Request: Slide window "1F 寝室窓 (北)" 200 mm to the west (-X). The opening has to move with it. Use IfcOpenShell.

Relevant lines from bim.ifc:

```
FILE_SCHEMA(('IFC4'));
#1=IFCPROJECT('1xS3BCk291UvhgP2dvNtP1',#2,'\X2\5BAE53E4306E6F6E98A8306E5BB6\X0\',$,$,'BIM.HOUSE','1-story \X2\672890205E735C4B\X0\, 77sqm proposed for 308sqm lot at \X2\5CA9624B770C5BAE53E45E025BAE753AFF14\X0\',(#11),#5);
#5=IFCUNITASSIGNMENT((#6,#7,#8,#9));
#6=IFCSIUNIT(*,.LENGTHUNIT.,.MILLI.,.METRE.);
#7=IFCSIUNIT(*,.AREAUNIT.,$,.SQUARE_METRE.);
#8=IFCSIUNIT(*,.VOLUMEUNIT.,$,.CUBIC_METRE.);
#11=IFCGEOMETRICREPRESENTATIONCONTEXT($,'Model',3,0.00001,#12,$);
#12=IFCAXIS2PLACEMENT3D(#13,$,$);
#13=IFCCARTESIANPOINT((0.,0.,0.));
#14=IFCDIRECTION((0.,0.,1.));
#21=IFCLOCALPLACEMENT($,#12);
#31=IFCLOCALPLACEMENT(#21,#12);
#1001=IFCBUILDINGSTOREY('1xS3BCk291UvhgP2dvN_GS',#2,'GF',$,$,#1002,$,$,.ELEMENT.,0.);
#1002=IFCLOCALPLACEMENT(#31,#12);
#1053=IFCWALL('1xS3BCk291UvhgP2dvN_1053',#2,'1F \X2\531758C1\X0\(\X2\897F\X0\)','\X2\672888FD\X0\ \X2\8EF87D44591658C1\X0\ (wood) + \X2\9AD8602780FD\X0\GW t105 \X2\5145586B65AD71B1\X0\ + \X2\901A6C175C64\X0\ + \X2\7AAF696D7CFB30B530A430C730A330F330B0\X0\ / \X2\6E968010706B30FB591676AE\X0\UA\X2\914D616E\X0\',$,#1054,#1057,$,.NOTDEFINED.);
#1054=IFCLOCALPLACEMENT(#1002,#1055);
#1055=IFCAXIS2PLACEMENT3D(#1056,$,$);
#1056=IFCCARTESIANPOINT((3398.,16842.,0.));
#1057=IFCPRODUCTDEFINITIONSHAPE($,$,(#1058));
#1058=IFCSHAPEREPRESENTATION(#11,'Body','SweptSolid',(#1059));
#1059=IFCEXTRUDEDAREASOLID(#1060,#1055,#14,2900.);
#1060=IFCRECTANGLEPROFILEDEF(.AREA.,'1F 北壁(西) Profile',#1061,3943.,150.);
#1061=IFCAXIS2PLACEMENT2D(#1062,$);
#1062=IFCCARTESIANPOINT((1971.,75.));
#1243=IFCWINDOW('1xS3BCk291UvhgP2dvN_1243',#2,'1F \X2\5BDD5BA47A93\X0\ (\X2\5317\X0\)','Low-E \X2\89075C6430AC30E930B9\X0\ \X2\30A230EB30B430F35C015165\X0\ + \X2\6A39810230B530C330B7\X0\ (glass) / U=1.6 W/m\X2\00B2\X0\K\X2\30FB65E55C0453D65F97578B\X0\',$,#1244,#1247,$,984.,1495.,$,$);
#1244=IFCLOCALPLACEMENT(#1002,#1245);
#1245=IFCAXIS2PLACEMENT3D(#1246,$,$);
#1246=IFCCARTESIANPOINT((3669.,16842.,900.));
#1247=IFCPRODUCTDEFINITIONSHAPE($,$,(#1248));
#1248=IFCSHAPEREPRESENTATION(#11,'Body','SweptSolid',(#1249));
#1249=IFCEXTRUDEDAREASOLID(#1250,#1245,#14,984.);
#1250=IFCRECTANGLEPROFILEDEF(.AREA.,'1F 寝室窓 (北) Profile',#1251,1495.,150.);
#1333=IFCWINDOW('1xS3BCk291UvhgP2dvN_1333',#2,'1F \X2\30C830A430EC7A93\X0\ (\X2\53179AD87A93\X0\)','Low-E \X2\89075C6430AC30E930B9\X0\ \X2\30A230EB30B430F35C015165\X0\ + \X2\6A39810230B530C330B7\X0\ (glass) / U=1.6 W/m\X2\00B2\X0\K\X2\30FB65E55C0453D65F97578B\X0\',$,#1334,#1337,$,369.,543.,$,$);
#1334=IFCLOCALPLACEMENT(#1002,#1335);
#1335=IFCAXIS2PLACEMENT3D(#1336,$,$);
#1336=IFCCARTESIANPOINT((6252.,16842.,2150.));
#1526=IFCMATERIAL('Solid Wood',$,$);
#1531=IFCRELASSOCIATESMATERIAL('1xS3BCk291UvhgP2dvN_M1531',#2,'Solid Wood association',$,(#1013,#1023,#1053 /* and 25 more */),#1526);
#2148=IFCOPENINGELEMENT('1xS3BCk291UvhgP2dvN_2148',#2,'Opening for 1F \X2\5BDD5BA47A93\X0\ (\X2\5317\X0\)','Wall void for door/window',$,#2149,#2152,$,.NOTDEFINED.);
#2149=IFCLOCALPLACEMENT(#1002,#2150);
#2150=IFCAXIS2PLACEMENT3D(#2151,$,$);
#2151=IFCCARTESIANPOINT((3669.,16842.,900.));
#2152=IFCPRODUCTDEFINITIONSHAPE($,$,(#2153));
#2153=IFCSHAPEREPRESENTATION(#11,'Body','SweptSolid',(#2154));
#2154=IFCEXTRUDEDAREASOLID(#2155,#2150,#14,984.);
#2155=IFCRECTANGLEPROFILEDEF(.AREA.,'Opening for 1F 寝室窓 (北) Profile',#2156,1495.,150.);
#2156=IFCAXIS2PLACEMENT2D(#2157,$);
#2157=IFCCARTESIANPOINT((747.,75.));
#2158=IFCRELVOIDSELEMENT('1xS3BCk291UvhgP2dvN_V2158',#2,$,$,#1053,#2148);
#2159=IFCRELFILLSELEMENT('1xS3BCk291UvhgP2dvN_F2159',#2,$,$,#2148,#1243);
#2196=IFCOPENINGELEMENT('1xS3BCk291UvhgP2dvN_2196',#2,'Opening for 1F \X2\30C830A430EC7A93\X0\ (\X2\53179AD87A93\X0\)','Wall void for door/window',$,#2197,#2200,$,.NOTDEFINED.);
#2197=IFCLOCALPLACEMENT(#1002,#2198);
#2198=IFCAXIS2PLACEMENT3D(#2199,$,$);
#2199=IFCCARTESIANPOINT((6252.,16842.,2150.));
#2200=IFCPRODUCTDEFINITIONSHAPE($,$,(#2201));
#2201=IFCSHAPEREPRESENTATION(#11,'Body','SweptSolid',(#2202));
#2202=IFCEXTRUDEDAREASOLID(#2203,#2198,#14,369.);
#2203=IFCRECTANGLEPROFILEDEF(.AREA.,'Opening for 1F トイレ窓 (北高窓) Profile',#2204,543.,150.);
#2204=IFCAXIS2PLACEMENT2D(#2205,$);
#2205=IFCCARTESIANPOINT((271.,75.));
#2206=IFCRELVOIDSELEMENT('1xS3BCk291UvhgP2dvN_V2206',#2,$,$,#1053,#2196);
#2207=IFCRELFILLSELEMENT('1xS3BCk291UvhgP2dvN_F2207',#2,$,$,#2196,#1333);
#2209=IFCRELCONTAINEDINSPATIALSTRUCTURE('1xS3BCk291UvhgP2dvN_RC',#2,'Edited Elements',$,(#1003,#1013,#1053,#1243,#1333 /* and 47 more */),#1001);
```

```python
import ifcopenshell
import ifcopenshell.api.geometry
import ifcopenshell.util.placement

model = ifcopenshell.open("bim.ifc")

window = model.by_guid("1xS3BCk291UvhgP2dvN_1243")
opening = window.FillsVoids[0].RelatingOpeningElement
wall = opening.VoidsElements[0].RelatingBuildingElement

wall_matrix = ifcopenshell.util.placement.get_local_placement(wall.ObjectPlacement)
shift = wall_matrix[:3, 0] * -200.0
before = ifcopenshell.util.placement.get_local_placement(window.ObjectPlacement)[:3, 3].copy()

# The window is not placed relative to its opening, so move both.
for product in (opening, window):
    matrix = ifcopenshell.util.placement.get_local_placement(product.ObjectPlacement)
    matrix[:3, 3] += shift
    ifcopenshell.api.geometry.edit_object_placement(model, product=product, matrix=matrix, is_si=False)

after = ifcopenshell.util.placement.get_local_placement(window.ObjectPlacement)[:3, 3]
print("window moved by", (after - before).round(3) + 0.0)

model.write("bim_rev.ifc")
```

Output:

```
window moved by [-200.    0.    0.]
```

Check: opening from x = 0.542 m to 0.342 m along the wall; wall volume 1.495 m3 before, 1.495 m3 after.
